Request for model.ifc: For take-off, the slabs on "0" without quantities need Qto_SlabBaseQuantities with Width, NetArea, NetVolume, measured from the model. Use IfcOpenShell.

First a look at what the model holds.

```python
import ifcopenshell
import ifcopenshell.util.element
import ifcopenshell.util.unit

model = ifcopenshell.open("model.ifc")
print(model.schema)
for unit_type in ("LENGTHUNIT", "AREAUNIT", "VOLUMEUNIT"):
    print(unit_type, ifcopenshell.util.unit.calculate_unit_scale(model, unit_type))
storey = next(s for s in model.by_type("IfcBuildingStorey") if s.Name == "0")
slabs = [e for e in ifcopenshell.util.element.get_decomposition(storey) if e.is_a("IfcSlab")]
for e in sorted(slabs, key=lambda e: e.id()):
    print(e.id(), e.is_a(), e.Name, list(ifcopenshell.util.element.get_psets(e, qtos_only=True)), sep=" | ")
```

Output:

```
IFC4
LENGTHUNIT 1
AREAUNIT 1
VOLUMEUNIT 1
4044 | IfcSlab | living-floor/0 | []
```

```python
import ifcopenshell
import ifcopenshell.api.pset
import ifcopenshell.geom
import ifcopenshell.util.element
import ifcopenshell.util.shape
import ifcopenshell.util.unit

model = ifcopenshell.open("model.ifc")
unit_scale = ifcopenshell.util.unit.calculate_unit_scale(model)
area_scale = ifcopenshell.util.unit.calculate_unit_scale(model, "AREAUNIT")
volume_scale = ifcopenshell.util.unit.calculate_unit_scale(model, "VOLUMEUNIT")
settings = ifcopenshell.geom.settings()

storey = next(s for s in model.by_type("IfcBuildingStorey") if s.Name == "0")
slabs = [e for e in ifcopenshell.util.element.get_decomposition(storey) if e.is_a("IfcSlab")]

for e in sorted(slabs, key=lambda e: e.id()):
    if ifcopenshell.util.element.get_psets(e, qtos_only=True, should_inherit=False):
        continue
    # Geometry comes back in metres, in the element's own axes.
    shape = ifcopenshell.geom.create_shape(settings, e)
    values = {
        "Width": ifcopenshell.util.shape.get_z(shape.geometry) / unit_scale,
        "NetArea": ifcopenshell.util.shape.get_footprint_area(shape.geometry) / area_scale,
        "NetVolume": ifcopenshell.util.shape.get_volume(shape.geometry) / volume_scale,
    }
    qto = ifcopenshell.api.pset.add_qto(model, product=e, name="Qto_SlabBaseQuantities")
    ifcopenshell.api.pset.edit_qto(model, qto=qto, properties=values)
    print(e.id(), {k: round(v, 3) for k, v in values.items()})

model.write("model_rev.ifc")
```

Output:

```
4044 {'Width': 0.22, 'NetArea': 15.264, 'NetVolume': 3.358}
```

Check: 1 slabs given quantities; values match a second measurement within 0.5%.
